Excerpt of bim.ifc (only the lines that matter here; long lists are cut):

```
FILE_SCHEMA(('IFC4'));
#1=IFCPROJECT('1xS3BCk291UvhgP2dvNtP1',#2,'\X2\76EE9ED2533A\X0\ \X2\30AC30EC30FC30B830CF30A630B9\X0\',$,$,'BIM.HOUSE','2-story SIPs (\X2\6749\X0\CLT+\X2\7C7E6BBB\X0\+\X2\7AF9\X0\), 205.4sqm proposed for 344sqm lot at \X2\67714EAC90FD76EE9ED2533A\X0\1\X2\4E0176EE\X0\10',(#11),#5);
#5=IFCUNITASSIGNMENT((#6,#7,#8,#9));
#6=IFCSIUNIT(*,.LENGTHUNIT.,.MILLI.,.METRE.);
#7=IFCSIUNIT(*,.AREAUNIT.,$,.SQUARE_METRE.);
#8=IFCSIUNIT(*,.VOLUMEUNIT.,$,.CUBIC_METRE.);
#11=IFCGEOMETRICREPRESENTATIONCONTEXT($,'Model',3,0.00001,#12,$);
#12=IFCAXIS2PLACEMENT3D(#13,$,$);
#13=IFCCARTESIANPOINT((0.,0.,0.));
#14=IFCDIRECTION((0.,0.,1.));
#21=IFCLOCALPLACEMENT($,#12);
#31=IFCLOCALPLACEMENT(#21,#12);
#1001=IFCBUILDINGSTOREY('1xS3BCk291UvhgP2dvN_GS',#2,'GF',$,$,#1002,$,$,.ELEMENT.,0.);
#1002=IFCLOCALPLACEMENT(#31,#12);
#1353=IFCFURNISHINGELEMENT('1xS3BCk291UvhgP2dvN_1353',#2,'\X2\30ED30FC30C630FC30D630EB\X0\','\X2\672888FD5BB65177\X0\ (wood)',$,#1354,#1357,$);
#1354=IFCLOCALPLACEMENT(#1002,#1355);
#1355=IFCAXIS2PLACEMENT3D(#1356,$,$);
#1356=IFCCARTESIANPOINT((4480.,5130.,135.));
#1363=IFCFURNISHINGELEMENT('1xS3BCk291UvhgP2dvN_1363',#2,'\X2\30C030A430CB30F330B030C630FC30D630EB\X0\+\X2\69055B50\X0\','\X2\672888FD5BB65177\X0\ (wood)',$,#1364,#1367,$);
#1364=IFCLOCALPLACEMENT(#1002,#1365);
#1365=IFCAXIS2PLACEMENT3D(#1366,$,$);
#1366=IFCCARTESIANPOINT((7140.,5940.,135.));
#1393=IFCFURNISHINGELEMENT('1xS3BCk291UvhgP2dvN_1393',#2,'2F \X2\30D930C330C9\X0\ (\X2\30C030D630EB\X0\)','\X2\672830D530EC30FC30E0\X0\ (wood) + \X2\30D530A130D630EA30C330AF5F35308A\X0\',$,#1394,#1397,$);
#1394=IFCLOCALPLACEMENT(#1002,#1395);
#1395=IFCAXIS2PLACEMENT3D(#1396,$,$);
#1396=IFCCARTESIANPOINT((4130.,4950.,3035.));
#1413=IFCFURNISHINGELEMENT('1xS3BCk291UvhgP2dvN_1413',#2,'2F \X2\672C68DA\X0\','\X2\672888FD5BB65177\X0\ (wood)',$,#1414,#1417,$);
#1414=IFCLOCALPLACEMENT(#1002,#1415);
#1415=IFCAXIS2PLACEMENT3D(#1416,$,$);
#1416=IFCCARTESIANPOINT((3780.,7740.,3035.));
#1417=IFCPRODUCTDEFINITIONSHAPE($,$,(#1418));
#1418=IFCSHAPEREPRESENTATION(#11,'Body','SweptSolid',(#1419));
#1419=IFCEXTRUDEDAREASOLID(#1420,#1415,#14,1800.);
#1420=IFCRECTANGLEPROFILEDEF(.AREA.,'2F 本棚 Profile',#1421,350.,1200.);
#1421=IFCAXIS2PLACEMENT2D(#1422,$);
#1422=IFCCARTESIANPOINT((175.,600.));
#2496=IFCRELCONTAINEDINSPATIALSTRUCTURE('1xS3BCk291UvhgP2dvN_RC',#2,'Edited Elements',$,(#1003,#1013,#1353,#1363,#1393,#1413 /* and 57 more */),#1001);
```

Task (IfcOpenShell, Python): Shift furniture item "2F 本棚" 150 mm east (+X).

```python
import ifcopenshell
import ifcopenshell.api.geometry
import ifcopenshell.util.placement
import ifcopenshell.util.unit

model = ifcopenshell.open("bim.ifc")
unit_scale = ifcopenshell.util.unit.calculate_unit_scale(model)

item = model.by_guid("1xS3BCk291UvhgP2dvN_1413")
matrix = ifcopenshell.util.placement.get_local_placement(item.ObjectPlacement)
matrix[0, 3] += 0.15 / unit_scale
ifcopenshell.api.geometry.edit_object_placement(model, product=item, matrix=matrix, is_si=False)

print(ifcopenshell.util.placement.get_local_placement(item.ObjectPlacement).round(3) + 0.0)

model.write("bim_rev.ifc")
```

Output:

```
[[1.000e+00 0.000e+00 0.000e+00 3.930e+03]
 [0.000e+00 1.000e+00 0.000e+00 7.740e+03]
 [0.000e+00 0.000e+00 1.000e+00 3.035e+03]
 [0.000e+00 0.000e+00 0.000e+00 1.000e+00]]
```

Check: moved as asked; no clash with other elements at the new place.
